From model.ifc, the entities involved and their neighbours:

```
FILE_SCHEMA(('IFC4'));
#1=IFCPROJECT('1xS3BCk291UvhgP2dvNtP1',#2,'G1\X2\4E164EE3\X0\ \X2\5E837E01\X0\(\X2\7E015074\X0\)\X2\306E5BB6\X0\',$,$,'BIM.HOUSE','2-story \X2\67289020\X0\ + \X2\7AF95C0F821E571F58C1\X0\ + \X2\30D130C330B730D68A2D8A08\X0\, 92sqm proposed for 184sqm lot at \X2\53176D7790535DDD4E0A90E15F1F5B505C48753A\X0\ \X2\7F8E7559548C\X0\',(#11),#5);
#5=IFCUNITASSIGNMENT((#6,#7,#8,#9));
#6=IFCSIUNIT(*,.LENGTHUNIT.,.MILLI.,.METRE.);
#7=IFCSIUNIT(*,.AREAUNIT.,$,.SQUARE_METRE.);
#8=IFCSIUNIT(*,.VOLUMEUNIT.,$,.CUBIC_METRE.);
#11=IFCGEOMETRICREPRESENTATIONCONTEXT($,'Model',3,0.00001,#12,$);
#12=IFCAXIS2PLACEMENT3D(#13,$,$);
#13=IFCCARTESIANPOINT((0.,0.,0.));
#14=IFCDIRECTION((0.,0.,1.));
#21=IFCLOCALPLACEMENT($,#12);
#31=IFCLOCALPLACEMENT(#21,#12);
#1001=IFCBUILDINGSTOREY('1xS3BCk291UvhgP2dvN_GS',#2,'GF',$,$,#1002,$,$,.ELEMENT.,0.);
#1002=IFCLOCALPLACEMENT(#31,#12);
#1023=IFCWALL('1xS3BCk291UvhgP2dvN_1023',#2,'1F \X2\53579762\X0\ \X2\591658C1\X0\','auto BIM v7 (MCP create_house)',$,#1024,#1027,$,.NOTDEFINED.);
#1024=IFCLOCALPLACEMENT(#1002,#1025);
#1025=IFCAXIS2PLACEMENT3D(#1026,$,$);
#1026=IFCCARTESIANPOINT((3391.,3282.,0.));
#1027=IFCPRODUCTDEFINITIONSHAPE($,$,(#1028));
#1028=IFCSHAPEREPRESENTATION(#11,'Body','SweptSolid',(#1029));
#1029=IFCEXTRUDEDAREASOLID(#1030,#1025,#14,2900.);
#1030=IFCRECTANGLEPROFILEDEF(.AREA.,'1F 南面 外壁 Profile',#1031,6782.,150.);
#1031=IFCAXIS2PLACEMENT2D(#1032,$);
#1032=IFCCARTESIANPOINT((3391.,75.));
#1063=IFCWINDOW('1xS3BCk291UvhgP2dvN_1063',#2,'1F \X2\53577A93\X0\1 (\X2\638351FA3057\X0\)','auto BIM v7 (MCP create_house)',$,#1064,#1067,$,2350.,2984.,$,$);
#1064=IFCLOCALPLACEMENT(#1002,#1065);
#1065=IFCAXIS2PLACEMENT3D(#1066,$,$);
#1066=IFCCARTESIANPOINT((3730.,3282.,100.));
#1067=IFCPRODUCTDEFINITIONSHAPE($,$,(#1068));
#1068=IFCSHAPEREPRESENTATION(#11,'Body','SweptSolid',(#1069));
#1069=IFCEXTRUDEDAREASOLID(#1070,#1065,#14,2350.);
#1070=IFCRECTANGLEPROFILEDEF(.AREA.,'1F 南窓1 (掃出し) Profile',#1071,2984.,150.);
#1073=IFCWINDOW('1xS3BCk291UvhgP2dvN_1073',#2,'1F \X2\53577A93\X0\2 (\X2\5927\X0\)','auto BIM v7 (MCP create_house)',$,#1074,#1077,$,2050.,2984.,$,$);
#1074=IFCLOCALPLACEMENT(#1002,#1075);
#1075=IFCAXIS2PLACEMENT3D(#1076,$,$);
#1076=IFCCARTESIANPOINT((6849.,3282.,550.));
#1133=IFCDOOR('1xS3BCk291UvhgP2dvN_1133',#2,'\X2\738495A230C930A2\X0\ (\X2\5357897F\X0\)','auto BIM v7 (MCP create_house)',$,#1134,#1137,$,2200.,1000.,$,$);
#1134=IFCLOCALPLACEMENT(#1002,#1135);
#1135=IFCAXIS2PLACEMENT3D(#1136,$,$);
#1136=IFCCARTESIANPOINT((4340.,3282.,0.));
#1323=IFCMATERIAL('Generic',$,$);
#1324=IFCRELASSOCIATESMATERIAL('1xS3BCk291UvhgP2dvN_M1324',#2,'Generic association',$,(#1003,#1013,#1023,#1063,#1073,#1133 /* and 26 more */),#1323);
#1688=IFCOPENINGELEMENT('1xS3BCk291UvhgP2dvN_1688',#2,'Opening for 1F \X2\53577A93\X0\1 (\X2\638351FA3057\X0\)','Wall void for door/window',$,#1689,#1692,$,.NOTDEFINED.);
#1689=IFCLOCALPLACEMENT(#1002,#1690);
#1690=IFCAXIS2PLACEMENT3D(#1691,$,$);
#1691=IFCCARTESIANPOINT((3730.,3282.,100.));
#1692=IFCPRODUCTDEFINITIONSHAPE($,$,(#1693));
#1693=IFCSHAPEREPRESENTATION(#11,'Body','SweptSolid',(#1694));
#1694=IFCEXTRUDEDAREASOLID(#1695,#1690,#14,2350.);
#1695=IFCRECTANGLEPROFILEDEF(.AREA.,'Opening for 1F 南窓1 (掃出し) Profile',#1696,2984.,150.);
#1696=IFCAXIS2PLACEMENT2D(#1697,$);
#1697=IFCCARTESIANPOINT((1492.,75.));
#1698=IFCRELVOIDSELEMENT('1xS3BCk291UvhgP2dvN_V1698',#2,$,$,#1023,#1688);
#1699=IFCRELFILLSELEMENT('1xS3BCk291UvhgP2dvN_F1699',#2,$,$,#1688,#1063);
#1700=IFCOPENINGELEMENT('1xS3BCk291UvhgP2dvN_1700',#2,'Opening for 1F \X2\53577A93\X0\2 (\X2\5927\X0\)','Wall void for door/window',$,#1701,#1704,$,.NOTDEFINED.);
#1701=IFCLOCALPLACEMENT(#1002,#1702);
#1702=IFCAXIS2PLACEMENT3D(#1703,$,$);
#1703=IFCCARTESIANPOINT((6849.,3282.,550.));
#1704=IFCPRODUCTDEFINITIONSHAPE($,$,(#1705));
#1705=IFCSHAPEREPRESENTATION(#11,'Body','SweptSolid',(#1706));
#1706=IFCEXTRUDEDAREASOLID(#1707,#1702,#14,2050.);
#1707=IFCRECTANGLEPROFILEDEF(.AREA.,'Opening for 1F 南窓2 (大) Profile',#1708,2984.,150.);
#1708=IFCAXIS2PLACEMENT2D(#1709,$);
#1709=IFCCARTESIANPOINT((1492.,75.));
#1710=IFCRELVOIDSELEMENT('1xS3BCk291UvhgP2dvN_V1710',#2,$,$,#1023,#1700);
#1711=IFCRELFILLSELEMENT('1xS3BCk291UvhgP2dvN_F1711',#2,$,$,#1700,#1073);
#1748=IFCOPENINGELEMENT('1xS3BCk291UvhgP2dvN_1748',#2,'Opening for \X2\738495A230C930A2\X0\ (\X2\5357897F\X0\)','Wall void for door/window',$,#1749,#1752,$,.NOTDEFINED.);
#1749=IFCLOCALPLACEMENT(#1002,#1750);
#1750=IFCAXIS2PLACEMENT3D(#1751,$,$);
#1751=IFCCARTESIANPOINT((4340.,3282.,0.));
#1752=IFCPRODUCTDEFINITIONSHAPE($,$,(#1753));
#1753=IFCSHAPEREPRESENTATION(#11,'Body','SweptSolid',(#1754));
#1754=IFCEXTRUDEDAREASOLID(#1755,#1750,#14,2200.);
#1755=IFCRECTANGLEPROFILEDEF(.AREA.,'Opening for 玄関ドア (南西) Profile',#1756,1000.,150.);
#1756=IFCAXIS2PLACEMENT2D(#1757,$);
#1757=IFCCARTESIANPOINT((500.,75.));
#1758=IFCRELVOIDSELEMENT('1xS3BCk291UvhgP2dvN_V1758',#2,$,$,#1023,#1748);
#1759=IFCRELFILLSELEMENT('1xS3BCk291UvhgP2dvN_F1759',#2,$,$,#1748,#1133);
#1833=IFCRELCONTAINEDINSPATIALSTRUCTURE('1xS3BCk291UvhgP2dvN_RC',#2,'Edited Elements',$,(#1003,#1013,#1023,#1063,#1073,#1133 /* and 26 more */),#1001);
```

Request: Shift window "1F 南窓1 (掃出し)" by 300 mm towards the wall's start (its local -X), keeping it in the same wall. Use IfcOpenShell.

```python
import ifcopenshell
import ifcopenshell.api.geometry
import ifcopenshell.util.placement

model = ifcopenshell.open("model.ifc")

window = model.by_guid("1xS3BCk291UvhgP2dvN_1063")
opening = window.FillsVoids[0].RelatingOpeningElement
wall = opening.VoidsElements[0].RelatingBuildingElement

wall_matrix = ifcopenshell.util.placement.get_local_placement(wall.ObjectPlacement)
shift = wall_matrix[:3, 0] * -300.0
before = ifcopenshell.util.placement.get_local_placement(window.ObjectPlacement)[:3, 3].copy()

# The window is not placed relative to its opening, so move both.
for product in (opening, window):
    matrix = ifcopenshell.util.placement.get_local_placement(product.ObjectPlacement)
    matrix[:3, 3] += shift
    ifcopenshell.api.geometry.edit_object_placement(model, product=product, matrix=matrix, is_si=False)

after = ifcopenshell.util.placement.get_local_placement(window.ObjectPlacement)[:3, 3]
print("window moved by", (after - before).round(3) + 0.0)

model.write("model_edited.ifc")
```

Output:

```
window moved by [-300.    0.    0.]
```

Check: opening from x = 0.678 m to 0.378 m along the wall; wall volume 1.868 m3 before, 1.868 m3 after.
